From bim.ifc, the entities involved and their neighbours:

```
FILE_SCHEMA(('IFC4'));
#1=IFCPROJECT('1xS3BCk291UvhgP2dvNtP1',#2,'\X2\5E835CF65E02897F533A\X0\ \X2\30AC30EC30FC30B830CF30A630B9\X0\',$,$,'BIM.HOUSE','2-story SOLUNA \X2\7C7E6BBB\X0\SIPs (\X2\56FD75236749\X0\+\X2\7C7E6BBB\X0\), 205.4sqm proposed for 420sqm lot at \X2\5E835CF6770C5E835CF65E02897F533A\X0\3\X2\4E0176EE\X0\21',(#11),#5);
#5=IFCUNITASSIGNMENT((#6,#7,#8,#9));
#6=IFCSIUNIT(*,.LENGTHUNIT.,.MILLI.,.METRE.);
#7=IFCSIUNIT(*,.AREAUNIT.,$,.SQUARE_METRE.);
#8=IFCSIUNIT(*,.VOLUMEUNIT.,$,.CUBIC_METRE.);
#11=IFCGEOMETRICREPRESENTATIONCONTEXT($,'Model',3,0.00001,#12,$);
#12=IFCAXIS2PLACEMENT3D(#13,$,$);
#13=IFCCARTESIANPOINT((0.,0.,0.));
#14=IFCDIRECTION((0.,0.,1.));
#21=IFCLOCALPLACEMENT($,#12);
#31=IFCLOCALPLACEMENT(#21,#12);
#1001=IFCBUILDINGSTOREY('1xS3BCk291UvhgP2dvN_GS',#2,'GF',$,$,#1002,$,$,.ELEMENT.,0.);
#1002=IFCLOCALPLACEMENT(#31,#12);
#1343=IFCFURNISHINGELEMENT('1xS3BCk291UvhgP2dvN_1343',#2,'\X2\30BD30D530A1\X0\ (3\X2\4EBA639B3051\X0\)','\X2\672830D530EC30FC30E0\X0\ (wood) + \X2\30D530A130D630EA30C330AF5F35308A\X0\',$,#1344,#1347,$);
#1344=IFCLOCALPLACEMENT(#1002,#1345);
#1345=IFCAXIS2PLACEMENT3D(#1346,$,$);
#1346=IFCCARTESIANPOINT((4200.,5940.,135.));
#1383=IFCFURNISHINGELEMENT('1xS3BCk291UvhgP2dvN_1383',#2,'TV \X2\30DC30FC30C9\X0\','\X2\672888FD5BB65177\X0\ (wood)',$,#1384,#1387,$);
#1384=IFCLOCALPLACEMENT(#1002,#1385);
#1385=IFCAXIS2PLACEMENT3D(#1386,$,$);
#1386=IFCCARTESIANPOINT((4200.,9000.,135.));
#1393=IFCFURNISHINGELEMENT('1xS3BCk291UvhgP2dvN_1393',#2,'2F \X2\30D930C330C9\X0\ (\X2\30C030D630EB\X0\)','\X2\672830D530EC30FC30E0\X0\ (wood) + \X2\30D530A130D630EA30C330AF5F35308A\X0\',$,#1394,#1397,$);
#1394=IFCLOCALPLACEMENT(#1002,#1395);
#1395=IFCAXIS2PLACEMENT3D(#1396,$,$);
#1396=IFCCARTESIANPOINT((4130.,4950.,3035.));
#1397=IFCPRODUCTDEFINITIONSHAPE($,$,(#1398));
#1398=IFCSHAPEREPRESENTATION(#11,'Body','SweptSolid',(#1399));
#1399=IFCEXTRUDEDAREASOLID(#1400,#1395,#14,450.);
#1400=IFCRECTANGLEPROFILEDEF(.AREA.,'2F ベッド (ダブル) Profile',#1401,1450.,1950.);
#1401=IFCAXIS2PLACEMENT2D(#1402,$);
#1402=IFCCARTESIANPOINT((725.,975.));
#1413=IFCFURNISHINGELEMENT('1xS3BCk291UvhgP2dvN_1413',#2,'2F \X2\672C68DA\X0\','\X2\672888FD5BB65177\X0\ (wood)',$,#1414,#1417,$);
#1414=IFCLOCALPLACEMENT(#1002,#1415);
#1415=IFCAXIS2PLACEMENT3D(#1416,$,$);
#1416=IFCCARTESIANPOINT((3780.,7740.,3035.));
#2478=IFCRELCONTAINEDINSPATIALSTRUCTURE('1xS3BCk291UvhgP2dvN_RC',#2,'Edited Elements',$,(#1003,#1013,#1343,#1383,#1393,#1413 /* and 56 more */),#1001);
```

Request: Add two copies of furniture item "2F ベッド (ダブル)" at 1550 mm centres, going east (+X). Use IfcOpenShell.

```python
import numpy as np
import ifcopenshell
import ifcopenshell.api.geometry
import ifcopenshell.api.root
import ifcopenshell.util.element
import ifcopenshell.util.placement

model = ifcopenshell.open("bim.ifc")


def reuse_history(source, copy):
    """copy_class also copies each property set's owner history, people and application; keep the originals."""
    for rel in copy.IsDefinedBy:
        if rel.is_a("IfcRelDefinesByProperties") and (history := rel.RelatingPropertyDefinition.OwnerHistory):
            rel.RelatingPropertyDefinition.OwnerHistory = source.OwnerHistory
            ifcopenshell.util.element.remove_deep2(model, history)


source = model.by_id(1393)
base = ifcopenshell.util.placement.get_local_placement(source.ObjectPlacement)
step = np.array([1.0, 0.0, 0.0]) * 1550.0

for i in range(1, 3):
    copy = ifcopenshell.api.root.copy_class(model, product=source)
    copy.Representation = ifcopenshell.util.element.copy_deep(
        model, source.Representation, exclude=["IfcGeometricRepresentationContext", "IfcRepresentationMap"]
    )
    reuse_history(source, copy)
    matrix = base.copy()
    matrix[:3, 3] += i * step
    print("added at", matrix[:3, 3].round(3) + 0.0)
    ifcopenshell.api.geometry.edit_object_placement(model, product=copy, matrix=matrix, is_si=False)

model.write("bim_v2.ifc")
```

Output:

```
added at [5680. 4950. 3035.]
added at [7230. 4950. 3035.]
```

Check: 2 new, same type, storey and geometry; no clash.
